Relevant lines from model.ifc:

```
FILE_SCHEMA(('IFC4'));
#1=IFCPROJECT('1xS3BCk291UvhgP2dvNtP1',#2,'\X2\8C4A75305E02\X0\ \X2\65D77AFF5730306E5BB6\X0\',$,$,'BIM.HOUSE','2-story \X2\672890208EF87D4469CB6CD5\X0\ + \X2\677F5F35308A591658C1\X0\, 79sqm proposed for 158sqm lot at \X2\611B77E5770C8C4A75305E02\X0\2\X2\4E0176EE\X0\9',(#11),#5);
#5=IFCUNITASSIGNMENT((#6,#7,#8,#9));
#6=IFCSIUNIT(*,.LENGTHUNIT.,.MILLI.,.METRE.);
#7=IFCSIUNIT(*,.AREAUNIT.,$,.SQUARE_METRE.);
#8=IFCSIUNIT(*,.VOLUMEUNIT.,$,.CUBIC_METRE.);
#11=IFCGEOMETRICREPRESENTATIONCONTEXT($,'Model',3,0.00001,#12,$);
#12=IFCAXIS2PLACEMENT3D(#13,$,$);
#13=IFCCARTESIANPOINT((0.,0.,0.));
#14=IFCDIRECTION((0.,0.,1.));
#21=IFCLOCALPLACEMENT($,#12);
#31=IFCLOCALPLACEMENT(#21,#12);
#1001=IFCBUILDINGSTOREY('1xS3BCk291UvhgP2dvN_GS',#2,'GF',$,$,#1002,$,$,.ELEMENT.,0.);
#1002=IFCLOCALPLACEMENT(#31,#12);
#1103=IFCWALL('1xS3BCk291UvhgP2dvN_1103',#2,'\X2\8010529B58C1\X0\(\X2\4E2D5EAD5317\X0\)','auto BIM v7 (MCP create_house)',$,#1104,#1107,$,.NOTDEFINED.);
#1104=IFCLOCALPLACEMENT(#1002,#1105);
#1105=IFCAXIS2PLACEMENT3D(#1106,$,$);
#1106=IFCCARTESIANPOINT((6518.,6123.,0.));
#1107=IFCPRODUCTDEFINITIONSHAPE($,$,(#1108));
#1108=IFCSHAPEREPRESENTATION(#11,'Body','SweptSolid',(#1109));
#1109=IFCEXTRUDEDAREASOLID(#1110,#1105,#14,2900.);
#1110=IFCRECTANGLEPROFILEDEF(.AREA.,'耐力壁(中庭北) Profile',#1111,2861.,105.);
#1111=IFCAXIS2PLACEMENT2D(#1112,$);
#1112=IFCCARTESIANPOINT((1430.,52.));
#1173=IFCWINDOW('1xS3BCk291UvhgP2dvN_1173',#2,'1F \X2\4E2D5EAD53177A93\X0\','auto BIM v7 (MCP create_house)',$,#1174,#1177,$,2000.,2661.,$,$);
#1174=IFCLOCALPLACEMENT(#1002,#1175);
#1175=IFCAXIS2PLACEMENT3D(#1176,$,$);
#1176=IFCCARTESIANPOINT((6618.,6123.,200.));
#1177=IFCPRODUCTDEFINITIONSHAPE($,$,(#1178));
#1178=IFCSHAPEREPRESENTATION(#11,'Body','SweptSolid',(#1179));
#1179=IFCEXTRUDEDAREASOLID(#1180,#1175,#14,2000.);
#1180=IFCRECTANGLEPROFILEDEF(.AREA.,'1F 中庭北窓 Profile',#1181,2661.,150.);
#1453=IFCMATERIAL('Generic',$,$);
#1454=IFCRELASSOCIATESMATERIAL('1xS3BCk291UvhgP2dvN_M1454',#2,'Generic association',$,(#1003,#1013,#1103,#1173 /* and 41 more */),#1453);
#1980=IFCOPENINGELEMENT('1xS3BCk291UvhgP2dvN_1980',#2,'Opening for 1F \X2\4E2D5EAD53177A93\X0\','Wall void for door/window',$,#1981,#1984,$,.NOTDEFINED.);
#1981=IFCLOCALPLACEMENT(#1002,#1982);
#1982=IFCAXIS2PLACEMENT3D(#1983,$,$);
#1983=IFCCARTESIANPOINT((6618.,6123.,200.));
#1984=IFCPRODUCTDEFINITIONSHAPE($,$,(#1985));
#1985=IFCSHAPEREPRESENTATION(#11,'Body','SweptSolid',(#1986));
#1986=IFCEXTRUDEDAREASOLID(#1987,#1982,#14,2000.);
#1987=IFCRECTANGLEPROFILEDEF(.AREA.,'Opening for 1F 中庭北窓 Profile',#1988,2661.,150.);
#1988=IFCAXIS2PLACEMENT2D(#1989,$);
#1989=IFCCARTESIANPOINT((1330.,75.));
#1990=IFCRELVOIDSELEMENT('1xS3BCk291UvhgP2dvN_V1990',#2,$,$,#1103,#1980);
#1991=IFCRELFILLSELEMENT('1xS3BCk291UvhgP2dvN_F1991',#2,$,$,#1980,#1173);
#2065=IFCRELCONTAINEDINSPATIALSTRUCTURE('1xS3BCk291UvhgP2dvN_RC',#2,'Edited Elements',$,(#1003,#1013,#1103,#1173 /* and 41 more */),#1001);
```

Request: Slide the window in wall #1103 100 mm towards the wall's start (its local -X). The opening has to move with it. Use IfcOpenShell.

```python
import ifcopenshell
import ifcopenshell.api.geometry
import ifcopenshell.util.placement
import ifcopenshell.util.unit

model = ifcopenshell.open("model.ifc")
unit_scale = ifcopenshell.util.unit.calculate_unit_scale(model)

window = model.by_id(1173)
opening = window.FillsVoids[0].RelatingOpeningElement
wall = opening.VoidsElements[0].RelatingBuildingElement

wall_matrix = ifcopenshell.util.placement.get_local_placement(wall.ObjectPlacement)
shift = wall_matrix[:3, 0] * -0.1 / unit_scale
before = ifcopenshell.util.placement.get_local_placement(window.ObjectPlacement)[:3, 3].copy()

# The window is not placed relative to its opening, so move both.
for product in (opening, window):
    matrix = ifcopenshell.util.placement.get_local_placement(product.ObjectPlacement)
    matrix[:3, 3] += shift
    ifcopenshell.api.geometry.edit_object_placement(model, product=product, matrix=matrix, is_si=False)

after = ifcopenshell.util.placement.get_local_placement(window.ObjectPlacement)[:3, 3]
print("window moved by", (after - before).round(3) + 0.0)

model.write("model_rev.ifc")
```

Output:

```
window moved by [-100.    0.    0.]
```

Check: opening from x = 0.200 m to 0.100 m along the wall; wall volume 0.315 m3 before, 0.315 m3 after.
